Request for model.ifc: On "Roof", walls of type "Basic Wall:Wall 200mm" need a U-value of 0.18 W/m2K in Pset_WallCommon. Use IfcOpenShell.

First a look at what the model holds.

```python
import ifcopenshell
import ifcopenshell.util.element

model = ifcopenshell.open("model.ifc")
print(model.schema)
storey = next(s for s in model.by_type("IfcBuildingStorey") if s.Name == "Roof")
walls = [e for e in ifcopenshell.util.element.get_decomposition(storey) if e.is_a("IfcWall")]
seen = {}
for e in walls:
    element_type = ifcopenshell.util.element.get_type(e)
    key = (element_type.Name if element_type != e and element_type else None, ifcopenshell.util.element.get_pset(e, "Pset_WallCommon", "ThermalTransmittance"))
    seen[key] = seen.get(key, 0) + 1
for (name, value), count in sorted(seen.items(), key=str):
    print(count, "x", name, "|", value)
```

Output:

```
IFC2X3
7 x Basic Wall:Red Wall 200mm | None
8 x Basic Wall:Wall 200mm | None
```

```python
import ifcopenshell
import ifcopenshell.api.pset
import ifcopenshell.util.element

model = ifcopenshell.open("model.ifc")

storey = next(s for s in model.by_type("IfcBuildingStorey") if s.Name == "Roof")
walls = [e for e in ifcopenshell.util.element.get_decomposition(storey) if e.is_a("IfcWall")]

count = 0
for e in walls:
    element_type = ifcopenshell.util.element.get_type(e)
    if element_type in (None, e) or element_type.Name != "Basic Wall:Wall 200mm":
        continue
    # add_pset returns the element's existing set when there is one.
    pset = ifcopenshell.api.pset.add_pset(model, product=e, name="Pset_WallCommon")
    ifcopenshell.api.pset.edit_pset(model, pset=pset, properties={"ThermalTransmittance": 0.18})
    count += 1

print(count, "walls updated")

model.write("model_v2.ifc")
```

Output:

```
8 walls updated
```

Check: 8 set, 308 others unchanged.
